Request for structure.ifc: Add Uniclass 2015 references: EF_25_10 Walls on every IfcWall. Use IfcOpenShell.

First a look at what the model holds.

```python
import ifcopenshell

model = ifcopenshell.open("structure.ifc")
print(model.schema)
print("classifications:", [c.Name for c in model.by_type("IfcClassification")])
for ifc_class in ("IfcDoor", "IfcRoof", "IfcStair", "IfcWall", "IfcWindow"):
    print(ifc_class, len(model.by_type(ifc_class)))
```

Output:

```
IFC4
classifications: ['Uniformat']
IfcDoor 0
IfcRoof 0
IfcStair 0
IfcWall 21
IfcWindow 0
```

```python
import ifcopenshell
import ifcopenshell.api.classification

model = ifcopenshell.open("structure.ifc")

system = ifcopenshell.api.classification.add_classification(model, classification="Uniclass 2015")

codes = {
    "IfcWall": ("EF_25_10", "Walls"),
}
for ifc_class, (code, name) in codes.items():
    products = model.by_type(ifc_class)
    ifcopenshell.api.classification.add_reference(
        model, products=products, classification=system, identification=code, name=name
    )
    print(code, len(products))

model.write("structure_rev.ifc")
```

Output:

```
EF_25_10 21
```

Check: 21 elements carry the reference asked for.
